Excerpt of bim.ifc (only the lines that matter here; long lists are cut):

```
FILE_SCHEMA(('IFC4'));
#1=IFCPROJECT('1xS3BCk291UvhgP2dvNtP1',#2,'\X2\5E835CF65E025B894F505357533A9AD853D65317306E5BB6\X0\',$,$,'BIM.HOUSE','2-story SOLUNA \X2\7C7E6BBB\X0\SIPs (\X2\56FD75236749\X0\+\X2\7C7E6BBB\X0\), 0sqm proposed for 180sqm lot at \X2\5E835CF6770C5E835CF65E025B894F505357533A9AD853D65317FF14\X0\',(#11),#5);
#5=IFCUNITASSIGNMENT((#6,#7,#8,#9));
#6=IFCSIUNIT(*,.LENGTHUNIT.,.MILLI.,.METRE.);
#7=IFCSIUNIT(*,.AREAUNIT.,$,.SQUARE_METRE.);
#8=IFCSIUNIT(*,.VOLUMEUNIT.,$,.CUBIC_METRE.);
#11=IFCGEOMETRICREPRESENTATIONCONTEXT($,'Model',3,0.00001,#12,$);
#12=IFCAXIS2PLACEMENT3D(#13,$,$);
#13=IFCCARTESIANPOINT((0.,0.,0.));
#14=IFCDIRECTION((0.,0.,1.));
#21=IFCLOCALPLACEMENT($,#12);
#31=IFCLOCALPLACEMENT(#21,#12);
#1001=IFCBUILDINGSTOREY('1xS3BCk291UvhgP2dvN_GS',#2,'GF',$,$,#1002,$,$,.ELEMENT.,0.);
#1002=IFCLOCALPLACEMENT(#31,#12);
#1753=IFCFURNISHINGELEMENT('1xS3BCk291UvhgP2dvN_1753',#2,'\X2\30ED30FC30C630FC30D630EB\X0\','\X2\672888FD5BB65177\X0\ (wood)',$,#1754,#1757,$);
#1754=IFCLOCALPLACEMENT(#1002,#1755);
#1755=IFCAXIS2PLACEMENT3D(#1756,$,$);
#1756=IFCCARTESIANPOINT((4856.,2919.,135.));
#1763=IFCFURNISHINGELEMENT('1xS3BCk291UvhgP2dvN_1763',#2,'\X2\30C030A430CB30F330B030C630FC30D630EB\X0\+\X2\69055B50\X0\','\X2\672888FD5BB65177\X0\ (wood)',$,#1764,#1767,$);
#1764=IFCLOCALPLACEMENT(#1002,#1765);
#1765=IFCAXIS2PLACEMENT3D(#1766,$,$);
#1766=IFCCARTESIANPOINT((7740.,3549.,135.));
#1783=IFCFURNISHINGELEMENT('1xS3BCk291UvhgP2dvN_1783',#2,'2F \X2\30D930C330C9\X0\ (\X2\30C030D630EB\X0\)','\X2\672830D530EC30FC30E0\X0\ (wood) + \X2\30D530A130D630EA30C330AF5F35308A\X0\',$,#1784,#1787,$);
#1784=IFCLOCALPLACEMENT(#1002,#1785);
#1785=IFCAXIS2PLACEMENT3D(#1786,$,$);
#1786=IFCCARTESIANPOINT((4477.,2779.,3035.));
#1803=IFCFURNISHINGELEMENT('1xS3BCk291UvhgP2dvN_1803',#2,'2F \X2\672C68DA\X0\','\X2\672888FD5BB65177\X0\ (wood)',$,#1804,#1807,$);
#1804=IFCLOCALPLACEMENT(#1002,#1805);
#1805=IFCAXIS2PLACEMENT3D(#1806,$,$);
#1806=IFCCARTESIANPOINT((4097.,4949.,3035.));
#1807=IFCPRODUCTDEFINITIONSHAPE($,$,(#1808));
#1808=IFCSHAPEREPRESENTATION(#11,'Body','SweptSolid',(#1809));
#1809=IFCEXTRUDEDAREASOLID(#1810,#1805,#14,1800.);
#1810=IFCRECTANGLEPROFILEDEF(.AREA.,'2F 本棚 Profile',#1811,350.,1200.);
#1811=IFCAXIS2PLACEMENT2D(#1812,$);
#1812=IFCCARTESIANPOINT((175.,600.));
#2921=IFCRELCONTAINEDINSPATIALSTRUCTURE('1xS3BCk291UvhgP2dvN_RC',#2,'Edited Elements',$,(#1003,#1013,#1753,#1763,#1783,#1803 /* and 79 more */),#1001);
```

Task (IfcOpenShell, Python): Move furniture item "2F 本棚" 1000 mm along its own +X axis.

```python
import ifcopenshell
import ifcopenshell.api.geometry
import ifcopenshell.util.placement

model = ifcopenshell.open("bim.ifc")

item = model.by_guid("1xS3BCk291UvhgP2dvN_1803")
matrix = ifcopenshell.util.placement.get_local_placement(item.ObjectPlacement)
matrix[:3, 3] += matrix[:3, 0] * 1000.0
ifcopenshell.api.geometry.edit_object_placement(model, product=item, matrix=matrix, is_si=False)

print(ifcopenshell.util.placement.get_local_placement(item.ObjectPlacement).round(3) + 0.0)

model.write("bim_updated.ifc")
```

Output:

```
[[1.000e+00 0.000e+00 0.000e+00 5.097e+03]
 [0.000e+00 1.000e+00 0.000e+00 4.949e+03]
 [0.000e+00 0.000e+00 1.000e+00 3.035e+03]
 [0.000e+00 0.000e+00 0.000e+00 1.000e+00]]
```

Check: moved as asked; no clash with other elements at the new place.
